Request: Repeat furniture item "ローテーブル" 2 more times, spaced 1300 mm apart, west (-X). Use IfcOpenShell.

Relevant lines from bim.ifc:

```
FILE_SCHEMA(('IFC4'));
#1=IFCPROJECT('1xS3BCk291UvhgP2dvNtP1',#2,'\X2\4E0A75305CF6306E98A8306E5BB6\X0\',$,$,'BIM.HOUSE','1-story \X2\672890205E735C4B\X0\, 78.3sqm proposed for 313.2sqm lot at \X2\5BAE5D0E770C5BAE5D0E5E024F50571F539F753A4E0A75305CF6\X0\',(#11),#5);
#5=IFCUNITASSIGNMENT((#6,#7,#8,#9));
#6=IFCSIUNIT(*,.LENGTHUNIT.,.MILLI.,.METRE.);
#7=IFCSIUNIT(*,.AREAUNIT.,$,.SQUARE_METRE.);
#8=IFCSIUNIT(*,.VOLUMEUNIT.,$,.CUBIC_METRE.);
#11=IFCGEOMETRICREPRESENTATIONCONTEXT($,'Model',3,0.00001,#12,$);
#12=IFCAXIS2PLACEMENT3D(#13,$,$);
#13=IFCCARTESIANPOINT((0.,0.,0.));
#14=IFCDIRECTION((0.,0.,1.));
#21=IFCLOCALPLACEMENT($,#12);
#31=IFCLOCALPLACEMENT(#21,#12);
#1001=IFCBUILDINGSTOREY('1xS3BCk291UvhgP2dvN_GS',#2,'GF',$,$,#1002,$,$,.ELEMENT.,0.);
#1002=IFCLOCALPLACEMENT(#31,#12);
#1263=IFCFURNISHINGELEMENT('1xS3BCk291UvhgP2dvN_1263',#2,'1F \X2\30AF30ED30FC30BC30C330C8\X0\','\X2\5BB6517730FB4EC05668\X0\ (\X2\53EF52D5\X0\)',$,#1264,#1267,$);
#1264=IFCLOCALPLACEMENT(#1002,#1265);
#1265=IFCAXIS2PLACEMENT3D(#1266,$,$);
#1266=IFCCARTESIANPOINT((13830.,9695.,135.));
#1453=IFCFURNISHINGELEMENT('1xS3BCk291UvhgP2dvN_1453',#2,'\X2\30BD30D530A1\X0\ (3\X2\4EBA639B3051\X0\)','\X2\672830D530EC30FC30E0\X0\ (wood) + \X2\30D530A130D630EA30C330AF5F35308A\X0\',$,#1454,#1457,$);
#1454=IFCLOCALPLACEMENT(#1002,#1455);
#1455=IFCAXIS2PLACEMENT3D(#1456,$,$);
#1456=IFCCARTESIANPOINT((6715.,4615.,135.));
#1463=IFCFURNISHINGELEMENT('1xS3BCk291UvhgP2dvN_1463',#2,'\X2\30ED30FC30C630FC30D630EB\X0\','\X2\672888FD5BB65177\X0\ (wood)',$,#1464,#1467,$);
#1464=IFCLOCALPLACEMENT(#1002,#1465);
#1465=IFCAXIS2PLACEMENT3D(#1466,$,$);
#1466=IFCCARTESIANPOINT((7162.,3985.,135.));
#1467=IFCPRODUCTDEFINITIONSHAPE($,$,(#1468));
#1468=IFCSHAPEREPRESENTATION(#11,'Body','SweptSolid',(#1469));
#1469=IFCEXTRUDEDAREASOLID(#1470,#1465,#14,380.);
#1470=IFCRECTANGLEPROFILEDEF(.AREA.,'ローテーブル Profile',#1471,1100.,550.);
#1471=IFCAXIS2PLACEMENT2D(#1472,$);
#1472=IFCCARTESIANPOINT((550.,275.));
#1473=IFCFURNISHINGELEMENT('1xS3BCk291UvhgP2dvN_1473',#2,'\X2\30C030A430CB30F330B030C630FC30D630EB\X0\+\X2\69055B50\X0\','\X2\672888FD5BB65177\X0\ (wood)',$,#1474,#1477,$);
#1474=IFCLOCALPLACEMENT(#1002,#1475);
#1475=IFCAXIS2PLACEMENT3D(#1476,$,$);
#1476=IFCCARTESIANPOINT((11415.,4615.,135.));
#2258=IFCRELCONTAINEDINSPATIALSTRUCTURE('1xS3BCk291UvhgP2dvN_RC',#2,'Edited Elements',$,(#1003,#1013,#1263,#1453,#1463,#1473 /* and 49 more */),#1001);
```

```python
import numpy as np
import ifcopenshell
import ifcopenshell.api.geometry
import ifcopenshell.api.root
import ifcopenshell.util.element
import ifcopenshell.util.placement

model = ifcopenshell.open("bim.ifc")


def reuse_history(source, copy):
    """copy_class also copies each property set's owner history, people and application; keep the originals."""
    for rel in copy.IsDefinedBy:
        if rel.is_a("IfcRelDefinesByProperties") and (history := rel.RelatingPropertyDefinition.OwnerHistory):
            rel.RelatingPropertyDefinition.OwnerHistory = source.OwnerHistory
            ifcopenshell.util.element.remove_deep2(model, history)


source = model.by_id(1463)
base = ifcopenshell.util.placement.get_local_placement(source.ObjectPlacement)
step = np.array([-1.0, 0.0, 0.0]) * 1300.0

for i in range(1, 3):
    copy = ifcopenshell.api.root.copy_class(model, product=source)
    copy.Representation = ifcopenshell.util.element.copy_deep(
        model, source.Representation, exclude=["IfcGeometricRepresentationContext", "IfcRepresentationMap"]
    )
    reuse_history(source, copy)
    matrix = base.copy()
    matrix[:3, 3] += i * step
    print("added at", matrix[:3, 3].round(3) + 0.0)
    ifcopenshell.api.geometry.edit_object_placement(model, product=copy, matrix=matrix, is_si=False)

model.write("bim_v2.ifc")
```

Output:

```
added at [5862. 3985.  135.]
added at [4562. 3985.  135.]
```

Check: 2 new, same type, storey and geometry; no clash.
